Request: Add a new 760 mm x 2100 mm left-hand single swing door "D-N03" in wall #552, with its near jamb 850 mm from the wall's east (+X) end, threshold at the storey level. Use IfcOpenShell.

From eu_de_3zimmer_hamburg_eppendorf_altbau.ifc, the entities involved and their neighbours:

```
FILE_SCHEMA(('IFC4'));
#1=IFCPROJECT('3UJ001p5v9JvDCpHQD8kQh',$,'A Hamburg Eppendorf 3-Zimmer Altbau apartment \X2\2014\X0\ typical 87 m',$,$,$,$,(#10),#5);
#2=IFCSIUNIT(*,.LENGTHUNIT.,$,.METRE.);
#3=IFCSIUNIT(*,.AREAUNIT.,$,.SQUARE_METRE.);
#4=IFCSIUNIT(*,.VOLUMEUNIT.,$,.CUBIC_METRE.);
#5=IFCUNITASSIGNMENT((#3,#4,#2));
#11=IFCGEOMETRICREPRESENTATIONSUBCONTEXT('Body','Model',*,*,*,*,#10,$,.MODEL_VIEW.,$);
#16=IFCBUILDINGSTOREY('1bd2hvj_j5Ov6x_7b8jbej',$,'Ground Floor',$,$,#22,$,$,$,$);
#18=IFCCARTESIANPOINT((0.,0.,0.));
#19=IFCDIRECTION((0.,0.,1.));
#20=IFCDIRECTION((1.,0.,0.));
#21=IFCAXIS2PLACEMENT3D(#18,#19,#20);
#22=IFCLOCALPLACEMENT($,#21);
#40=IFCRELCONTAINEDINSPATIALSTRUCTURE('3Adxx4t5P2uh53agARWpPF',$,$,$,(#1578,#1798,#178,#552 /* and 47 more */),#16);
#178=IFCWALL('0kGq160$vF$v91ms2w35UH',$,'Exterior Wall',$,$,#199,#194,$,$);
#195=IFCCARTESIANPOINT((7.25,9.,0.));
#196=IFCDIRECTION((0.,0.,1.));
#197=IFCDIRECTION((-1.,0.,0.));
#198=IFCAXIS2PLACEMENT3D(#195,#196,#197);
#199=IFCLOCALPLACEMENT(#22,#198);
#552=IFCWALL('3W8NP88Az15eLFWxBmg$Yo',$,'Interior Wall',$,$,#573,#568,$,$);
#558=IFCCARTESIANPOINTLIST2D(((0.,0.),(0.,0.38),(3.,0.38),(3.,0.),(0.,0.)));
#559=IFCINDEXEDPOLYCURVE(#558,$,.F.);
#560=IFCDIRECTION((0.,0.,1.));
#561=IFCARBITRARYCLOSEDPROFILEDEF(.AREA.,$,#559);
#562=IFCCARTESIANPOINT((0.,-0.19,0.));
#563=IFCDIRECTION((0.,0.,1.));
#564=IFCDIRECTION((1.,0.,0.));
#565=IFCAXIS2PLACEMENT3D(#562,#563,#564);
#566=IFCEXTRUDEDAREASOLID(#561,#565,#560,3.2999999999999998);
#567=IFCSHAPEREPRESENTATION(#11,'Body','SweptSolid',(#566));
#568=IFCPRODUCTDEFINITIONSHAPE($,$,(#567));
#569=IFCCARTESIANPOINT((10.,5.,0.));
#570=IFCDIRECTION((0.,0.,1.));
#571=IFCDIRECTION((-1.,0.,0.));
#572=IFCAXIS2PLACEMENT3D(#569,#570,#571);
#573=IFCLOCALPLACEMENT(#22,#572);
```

```python
import numpy as np
import ifcopenshell
import ifcopenshell.api.feature
import ifcopenshell.api.geometry
import ifcopenshell.api.root
import ifcopenshell.api.spatial
import ifcopenshell.geom
import ifcopenshell.util.element
import ifcopenshell.util.placement
import ifcopenshell.util.representation
import ifcopenshell.util.shape
import ifcopenshell.util.unit

model = ifcopenshell.open("eu_de_3zimmer_hamburg_eppendorf_altbau.ifc")
unit_scale = ifcopenshell.util.unit.calculate_unit_scale(model)
settings = ifcopenshell.geom.settings()


def volume(element):
    """Net volume in cubic metres, openings subtracted."""
    shape = ifcopenshell.geom.create_shape(settings, element)
    return ifcopenshell.util.shape.get_volume(shape.geometry)


wall = model.by_guid("3W8NP88Az15eLFWxBmg$Yo")
storey = ifcopenshell.util.element.get_container(wall, ifc_class="IfcBuildingStorey")
context = ifcopenshell.util.representation.get_context(model, "Model", "Body", "MODEL_VIEW")
before = volume(wall)

width, height, from_end, sill = 0.76, 2.1, 0.85, 0.0  # metres

# The wall runs along its own X axis, and the end named is its -X end.
wall_shape = ifcopenshell.geom.create_shape(settings, wall)
x, y, z = ifcopenshell.util.shape.get_vertices(wall_shape.geometry).T
start = x.min() + from_end
face, thickness = float(y.min()), float(y.max() - y.min())
wall_matrix = ifcopenshell.util.placement.get_local_placement(wall.ObjectPlacement)
level = ifcopenshell.util.placement.get_local_placement(storey.ObjectPlacement)[2, 3]


def in_wall(x, y):
    """Placement at x, y metres in the wall's axes, at sill height."""
    matrix = wall_matrix.copy()
    matrix[:, 3] = wall_matrix @ np.array([x / unit_scale, y / unit_scale, 0.0, 1.0])
    matrix[2, 3] = level + sill / unit_scale
    return matrix


# Opening: a box that overshoots both wall faces by 50 mm.
opening = ifcopenshell.api.root.create_entity(model, ifc_class="IfcOpeningElement", predefined_type="OPENING")
box = ifcopenshell.api.geometry.add_wall_representation(
    model, context=context, length=width, height=height, thickness=thickness + 0.1
)
ifcopenshell.api.geometry.assign_representation(model, product=opening, representation=box)
ifcopenshell.api.geometry.edit_object_placement(model, product=opening, matrix=in_wall(start, face - 0.05), is_si=False)
ifcopenshell.api.feature.add_feature(model, feature=opening, element=wall)

door = ifcopenshell.api.root.create_entity(model, ifc_class="IfcDoor", name="D-N03", predefined_type="DOOR")
door.OverallWidth, door.OverallHeight = width / unit_scale, height / unit_scale
door.OperationType = "SINGLE_SWING_LEFT"
body = ifcopenshell.api.geometry.add_door_representation(
    model,
    context=context,
    overall_width=door.OverallWidth,
    overall_height=door.OverallHeight,
    operation_type="SINGLE_SWING_LEFT",
    lining_properties={"LiningDepth": thickness / unit_scale, "ThresholdDepth": thickness / unit_scale},
)
ifcopenshell.api.geometry.assign_representation(model, product=door, representation=body)
ifcopenshell.api.spatial.assign_container(model, products=[door], relating_structure=storey)
ifcopenshell.api.feature.add_filling(model, opening=opening, element=door)

# The lining spans the wall, so the door starts at the wall face.
ifcopenshell.api.geometry.edit_object_placement(model, product=door, matrix=in_wall(start, face), is_si=False)

after = volume(wall)

print(f"wall volume {before:.3f} -> {after:.3f} m3")

model.write("eu_de_3zimmer_hamburg_eppendorf_altbau_v2.ifc")
```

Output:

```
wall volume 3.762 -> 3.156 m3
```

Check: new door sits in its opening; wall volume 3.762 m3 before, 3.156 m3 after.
